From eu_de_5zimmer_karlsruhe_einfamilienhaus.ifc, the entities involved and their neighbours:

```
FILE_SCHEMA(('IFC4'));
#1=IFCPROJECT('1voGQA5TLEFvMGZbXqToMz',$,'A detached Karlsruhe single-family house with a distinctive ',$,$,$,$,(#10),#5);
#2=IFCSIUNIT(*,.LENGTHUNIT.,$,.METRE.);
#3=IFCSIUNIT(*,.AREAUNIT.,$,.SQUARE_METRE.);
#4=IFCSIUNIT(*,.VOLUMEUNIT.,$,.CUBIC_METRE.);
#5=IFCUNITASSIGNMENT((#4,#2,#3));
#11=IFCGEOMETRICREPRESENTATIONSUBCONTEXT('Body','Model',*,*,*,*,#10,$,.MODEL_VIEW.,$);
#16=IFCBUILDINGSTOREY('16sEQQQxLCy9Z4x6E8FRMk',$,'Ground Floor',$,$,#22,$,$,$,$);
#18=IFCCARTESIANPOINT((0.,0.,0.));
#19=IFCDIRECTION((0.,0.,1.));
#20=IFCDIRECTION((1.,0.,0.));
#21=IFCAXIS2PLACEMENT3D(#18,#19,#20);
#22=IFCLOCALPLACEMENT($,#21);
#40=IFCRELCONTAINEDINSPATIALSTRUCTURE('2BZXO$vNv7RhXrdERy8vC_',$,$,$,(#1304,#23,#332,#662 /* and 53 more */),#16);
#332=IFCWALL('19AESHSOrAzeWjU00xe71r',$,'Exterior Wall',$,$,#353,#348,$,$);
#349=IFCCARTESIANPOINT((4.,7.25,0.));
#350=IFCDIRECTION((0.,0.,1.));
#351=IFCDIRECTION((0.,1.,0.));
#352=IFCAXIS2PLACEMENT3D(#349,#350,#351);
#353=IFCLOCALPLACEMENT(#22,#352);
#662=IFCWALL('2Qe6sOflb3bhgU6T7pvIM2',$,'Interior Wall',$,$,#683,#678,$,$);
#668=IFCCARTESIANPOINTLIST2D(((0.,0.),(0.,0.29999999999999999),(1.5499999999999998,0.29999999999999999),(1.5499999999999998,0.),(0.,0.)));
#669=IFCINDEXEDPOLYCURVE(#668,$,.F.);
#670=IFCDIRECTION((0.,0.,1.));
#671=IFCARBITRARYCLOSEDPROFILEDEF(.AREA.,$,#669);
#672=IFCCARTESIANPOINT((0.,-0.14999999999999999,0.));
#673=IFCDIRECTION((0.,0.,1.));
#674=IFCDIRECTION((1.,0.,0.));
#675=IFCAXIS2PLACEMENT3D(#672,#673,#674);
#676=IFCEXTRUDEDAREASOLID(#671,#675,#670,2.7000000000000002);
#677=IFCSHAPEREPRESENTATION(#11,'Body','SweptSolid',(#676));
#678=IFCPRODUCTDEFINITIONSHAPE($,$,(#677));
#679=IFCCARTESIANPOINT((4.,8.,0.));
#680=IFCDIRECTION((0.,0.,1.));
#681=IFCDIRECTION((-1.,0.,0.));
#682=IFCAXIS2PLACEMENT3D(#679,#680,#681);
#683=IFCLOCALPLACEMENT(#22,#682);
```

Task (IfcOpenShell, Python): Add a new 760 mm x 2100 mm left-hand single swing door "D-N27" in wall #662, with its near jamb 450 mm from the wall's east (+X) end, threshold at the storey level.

```python
import numpy as np
import ifcopenshell
import ifcopenshell.api.feature
import ifcopenshell.api.geometry
import ifcopenshell.api.root
import ifcopenshell.api.spatial
import ifcopenshell.geom
import ifcopenshell.util.element
import ifcopenshell.util.placement
import ifcopenshell.util.representation
import ifcopenshell.util.shape
import ifcopenshell.util.unit

model = ifcopenshell.open("eu_de_5zimmer_karlsruhe_einfamilienhaus.ifc")
unit_scale = ifcopenshell.util.unit.calculate_unit_scale(model)
settings = ifcopenshell.geom.settings()


def volume(element):
    """Net volume in cubic metres, openings subtracted."""
    shape = ifcopenshell.geom.create_shape(settings, element)
    return ifcopenshell.util.shape.get_volume(shape.geometry)


wall = model.by_guid("2Qe6sOflb3bhgU6T7pvIM2")
storey = ifcopenshell.util.element.get_container(wall, ifc_class="IfcBuildingStorey")
context = ifcopenshell.util.representation.get_context(model, "Model", "Body", "MODEL_VIEW")
before = volume(wall)

width, height, from_end, sill = 0.76, 2.1, 0.45, 0.0  # metres

# The wall runs along its own X axis, and the end named is its -X end.
wall_shape = ifcopenshell.geom.create_shape(settings, wall)
x, y, z = ifcopenshell.util.shape.get_vertices(wall_shape.geometry).T
start = x.min() + from_end
face, thickness = float(y.min()), float(y.max() - y.min())
wall_matrix = ifcopenshell.util.placement.get_local_placement(wall.ObjectPlacement)
level = ifcopenshell.util.placement.get_local_placement(storey.ObjectPlacement)[2, 3]


def in_wall(x, y):
    """Placement at x, y metres in the wall's axes, at sill height."""
    matrix = wall_matrix.copy()
    matrix[:, 3] = wall_matrix @ np.array([x / unit_scale, y / unit_scale, 0.0, 1.0])
    matrix[2, 3] = level + sill / unit_scale
    return matrix


# Opening: a box that overshoots both wall faces by 50 mm.
opening = ifcopenshell.api.root.create_entity(model, ifc_class="IfcOpeningElement", predefined_type="OPENING")
box = ifcopenshell.api.geometry.add_wall_representation(
    model, context=context, length=width, height=height, thickness=thickness + 0.1
)
ifcopenshell.api.geometry.assign_representation(model, product=opening, representation=box)
ifcopenshell.api.geometry.edit_object_placement(model, product=opening, matrix=in_wall(start, face - 0.05), is_si=False)
ifcopenshell.api.feature.add_feature(model, feature=opening, element=wall)

door = ifcopenshell.api.root.create_entity(model, ifc_class="IfcDoor", name="D-N27", predefined_type="DOOR")
door.OverallWidth, door.OverallHeight = width / unit_scale, height / unit_scale
door.OperationType = "SINGLE_SWING_LEFT"
body = ifcopenshell.api.geometry.add_door_representation(
    model,
    context=context,
    overall_width=door.OverallWidth,
    overall_height=door.OverallHeight,
    operation_type="SINGLE_SWING_LEFT",
    lining_properties={"LiningDepth": thickness / unit_scale, "ThresholdDepth": thickness / unit_scale},
)
ifcopenshell.api.geometry.assign_representation(model, product=door, representation=body)
ifcopenshell.api.spatial.assign_container(model, products=[door], relating_structure=storey)
ifcopenshell.api.feature.add_filling(model, opening=opening, element=door)

# The lining spans the wall, so the door starts at the wall face.
ifcopenshell.api.geometry.edit_object_placement(model, product=door, matrix=in_wall(start, face), is_si=False)

after = volume(wall)

print(f"wall volume {before:.3f} -> {after:.3f} m3")

model.write("eu_de_5zimmer_karlsruhe_einfamilienhaus_updated.ifc")
```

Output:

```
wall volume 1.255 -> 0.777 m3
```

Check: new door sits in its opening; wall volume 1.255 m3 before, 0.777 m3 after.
